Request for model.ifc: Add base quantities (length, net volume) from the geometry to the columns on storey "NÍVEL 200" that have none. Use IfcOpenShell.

First a look at what the model holds.

```python
import ifcopenshell
import ifcopenshell.util.element
import ifcopenshell.util.unit

model = ifcopenshell.open("model.ifc")
print(model.schema)
for unit_type in ("LENGTHUNIT", "AREAUNIT", "VOLUMEUNIT"):
    print(unit_type, ifcopenshell.util.unit.calculate_unit_scale(model, unit_type))
storey = next(s for s in model.by_type("IfcBuildingStorey") if s.Name == "NÍVEL 200")
columns = [e for e in ifcopenshell.util.element.get_decomposition(storey) if e.is_a("IfcColumn")]
for e in sorted(columns, key=lambda e: e.id()):
    print(e.id(), e.is_a(), e.Name, list(ifcopenshell.util.element.get_psets(e, qtos_only=True)), sep=" | ")
```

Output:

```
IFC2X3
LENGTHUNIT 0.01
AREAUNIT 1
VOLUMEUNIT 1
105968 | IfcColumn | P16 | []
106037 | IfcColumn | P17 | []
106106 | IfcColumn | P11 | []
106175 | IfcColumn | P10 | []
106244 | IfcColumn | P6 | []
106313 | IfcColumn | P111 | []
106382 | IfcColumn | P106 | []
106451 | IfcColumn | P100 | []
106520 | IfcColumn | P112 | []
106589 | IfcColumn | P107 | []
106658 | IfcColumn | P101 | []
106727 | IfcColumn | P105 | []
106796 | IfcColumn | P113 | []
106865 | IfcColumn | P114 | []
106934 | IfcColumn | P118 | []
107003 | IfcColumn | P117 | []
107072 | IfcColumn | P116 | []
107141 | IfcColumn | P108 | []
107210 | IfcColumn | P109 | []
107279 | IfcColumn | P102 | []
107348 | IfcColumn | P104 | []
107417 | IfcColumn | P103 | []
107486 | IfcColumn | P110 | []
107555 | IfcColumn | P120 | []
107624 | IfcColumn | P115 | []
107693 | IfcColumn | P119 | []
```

```python
import ifcopenshell
import ifcopenshell.api.pset
import ifcopenshell.geom
import ifcopenshell.util.element
import ifcopenshell.util.shape
import ifcopenshell.util.unit

model = ifcopenshell.open("model.ifc")
unit_scale = ifcopenshell.util.unit.calculate_unit_scale(model)
volume_scale = ifcopenshell.util.unit.calculate_unit_scale(model, "VOLUMEUNIT")
settings = ifcopenshell.geom.settings()

storey = next(s for s in model.by_type("IfcBuildingStorey") if s.Name == "NÍVEL 200")
columns = [e for e in ifcopenshell.util.element.get_decomposition(storey) if e.is_a("IfcColumn")]

for e in sorted(columns, key=lambda e: e.id()):
    if ifcopenshell.util.element.get_psets(e, qtos_only=True, should_inherit=False):
        continue
    # Geometry comes back in metres, in the element's own axes.
    shape = ifcopenshell.geom.create_shape(settings, e)
    values = {
        "Length": ifcopenshell.util.shape.get_z(shape.geometry) / unit_scale,
        "NetVolume": ifcopenshell.util.shape.get_volume(shape.geometry) / volume_scale,
    }
    qto = ifcopenshell.api.pset.add_qto(model, product=e, name="BaseQuantities")
    ifcopenshell.api.pset.edit_qto(model, qto=qto, properties=values)
    print(e.id(), {k: round(v, 3) for k, v in values.items()})

model.write("model_rev.ifc")
```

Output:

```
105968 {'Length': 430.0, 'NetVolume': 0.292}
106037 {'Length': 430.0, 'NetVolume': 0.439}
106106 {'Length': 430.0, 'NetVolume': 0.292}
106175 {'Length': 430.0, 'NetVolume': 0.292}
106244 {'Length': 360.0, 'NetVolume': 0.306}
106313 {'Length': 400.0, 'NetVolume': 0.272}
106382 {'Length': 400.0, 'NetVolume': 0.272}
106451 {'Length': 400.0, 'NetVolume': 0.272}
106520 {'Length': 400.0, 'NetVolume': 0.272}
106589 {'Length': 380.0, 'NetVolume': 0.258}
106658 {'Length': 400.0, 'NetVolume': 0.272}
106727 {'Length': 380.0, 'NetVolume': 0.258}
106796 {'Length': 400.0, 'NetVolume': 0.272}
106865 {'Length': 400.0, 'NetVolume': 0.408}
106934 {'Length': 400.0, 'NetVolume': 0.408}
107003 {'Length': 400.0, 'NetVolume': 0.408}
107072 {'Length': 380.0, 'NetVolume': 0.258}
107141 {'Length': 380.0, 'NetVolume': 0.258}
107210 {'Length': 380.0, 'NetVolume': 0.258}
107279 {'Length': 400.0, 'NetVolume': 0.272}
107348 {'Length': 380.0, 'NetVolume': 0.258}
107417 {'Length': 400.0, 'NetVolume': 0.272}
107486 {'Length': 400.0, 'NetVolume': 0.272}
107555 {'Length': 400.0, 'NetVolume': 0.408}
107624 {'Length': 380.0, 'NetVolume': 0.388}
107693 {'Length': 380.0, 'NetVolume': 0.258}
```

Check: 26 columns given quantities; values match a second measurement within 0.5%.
